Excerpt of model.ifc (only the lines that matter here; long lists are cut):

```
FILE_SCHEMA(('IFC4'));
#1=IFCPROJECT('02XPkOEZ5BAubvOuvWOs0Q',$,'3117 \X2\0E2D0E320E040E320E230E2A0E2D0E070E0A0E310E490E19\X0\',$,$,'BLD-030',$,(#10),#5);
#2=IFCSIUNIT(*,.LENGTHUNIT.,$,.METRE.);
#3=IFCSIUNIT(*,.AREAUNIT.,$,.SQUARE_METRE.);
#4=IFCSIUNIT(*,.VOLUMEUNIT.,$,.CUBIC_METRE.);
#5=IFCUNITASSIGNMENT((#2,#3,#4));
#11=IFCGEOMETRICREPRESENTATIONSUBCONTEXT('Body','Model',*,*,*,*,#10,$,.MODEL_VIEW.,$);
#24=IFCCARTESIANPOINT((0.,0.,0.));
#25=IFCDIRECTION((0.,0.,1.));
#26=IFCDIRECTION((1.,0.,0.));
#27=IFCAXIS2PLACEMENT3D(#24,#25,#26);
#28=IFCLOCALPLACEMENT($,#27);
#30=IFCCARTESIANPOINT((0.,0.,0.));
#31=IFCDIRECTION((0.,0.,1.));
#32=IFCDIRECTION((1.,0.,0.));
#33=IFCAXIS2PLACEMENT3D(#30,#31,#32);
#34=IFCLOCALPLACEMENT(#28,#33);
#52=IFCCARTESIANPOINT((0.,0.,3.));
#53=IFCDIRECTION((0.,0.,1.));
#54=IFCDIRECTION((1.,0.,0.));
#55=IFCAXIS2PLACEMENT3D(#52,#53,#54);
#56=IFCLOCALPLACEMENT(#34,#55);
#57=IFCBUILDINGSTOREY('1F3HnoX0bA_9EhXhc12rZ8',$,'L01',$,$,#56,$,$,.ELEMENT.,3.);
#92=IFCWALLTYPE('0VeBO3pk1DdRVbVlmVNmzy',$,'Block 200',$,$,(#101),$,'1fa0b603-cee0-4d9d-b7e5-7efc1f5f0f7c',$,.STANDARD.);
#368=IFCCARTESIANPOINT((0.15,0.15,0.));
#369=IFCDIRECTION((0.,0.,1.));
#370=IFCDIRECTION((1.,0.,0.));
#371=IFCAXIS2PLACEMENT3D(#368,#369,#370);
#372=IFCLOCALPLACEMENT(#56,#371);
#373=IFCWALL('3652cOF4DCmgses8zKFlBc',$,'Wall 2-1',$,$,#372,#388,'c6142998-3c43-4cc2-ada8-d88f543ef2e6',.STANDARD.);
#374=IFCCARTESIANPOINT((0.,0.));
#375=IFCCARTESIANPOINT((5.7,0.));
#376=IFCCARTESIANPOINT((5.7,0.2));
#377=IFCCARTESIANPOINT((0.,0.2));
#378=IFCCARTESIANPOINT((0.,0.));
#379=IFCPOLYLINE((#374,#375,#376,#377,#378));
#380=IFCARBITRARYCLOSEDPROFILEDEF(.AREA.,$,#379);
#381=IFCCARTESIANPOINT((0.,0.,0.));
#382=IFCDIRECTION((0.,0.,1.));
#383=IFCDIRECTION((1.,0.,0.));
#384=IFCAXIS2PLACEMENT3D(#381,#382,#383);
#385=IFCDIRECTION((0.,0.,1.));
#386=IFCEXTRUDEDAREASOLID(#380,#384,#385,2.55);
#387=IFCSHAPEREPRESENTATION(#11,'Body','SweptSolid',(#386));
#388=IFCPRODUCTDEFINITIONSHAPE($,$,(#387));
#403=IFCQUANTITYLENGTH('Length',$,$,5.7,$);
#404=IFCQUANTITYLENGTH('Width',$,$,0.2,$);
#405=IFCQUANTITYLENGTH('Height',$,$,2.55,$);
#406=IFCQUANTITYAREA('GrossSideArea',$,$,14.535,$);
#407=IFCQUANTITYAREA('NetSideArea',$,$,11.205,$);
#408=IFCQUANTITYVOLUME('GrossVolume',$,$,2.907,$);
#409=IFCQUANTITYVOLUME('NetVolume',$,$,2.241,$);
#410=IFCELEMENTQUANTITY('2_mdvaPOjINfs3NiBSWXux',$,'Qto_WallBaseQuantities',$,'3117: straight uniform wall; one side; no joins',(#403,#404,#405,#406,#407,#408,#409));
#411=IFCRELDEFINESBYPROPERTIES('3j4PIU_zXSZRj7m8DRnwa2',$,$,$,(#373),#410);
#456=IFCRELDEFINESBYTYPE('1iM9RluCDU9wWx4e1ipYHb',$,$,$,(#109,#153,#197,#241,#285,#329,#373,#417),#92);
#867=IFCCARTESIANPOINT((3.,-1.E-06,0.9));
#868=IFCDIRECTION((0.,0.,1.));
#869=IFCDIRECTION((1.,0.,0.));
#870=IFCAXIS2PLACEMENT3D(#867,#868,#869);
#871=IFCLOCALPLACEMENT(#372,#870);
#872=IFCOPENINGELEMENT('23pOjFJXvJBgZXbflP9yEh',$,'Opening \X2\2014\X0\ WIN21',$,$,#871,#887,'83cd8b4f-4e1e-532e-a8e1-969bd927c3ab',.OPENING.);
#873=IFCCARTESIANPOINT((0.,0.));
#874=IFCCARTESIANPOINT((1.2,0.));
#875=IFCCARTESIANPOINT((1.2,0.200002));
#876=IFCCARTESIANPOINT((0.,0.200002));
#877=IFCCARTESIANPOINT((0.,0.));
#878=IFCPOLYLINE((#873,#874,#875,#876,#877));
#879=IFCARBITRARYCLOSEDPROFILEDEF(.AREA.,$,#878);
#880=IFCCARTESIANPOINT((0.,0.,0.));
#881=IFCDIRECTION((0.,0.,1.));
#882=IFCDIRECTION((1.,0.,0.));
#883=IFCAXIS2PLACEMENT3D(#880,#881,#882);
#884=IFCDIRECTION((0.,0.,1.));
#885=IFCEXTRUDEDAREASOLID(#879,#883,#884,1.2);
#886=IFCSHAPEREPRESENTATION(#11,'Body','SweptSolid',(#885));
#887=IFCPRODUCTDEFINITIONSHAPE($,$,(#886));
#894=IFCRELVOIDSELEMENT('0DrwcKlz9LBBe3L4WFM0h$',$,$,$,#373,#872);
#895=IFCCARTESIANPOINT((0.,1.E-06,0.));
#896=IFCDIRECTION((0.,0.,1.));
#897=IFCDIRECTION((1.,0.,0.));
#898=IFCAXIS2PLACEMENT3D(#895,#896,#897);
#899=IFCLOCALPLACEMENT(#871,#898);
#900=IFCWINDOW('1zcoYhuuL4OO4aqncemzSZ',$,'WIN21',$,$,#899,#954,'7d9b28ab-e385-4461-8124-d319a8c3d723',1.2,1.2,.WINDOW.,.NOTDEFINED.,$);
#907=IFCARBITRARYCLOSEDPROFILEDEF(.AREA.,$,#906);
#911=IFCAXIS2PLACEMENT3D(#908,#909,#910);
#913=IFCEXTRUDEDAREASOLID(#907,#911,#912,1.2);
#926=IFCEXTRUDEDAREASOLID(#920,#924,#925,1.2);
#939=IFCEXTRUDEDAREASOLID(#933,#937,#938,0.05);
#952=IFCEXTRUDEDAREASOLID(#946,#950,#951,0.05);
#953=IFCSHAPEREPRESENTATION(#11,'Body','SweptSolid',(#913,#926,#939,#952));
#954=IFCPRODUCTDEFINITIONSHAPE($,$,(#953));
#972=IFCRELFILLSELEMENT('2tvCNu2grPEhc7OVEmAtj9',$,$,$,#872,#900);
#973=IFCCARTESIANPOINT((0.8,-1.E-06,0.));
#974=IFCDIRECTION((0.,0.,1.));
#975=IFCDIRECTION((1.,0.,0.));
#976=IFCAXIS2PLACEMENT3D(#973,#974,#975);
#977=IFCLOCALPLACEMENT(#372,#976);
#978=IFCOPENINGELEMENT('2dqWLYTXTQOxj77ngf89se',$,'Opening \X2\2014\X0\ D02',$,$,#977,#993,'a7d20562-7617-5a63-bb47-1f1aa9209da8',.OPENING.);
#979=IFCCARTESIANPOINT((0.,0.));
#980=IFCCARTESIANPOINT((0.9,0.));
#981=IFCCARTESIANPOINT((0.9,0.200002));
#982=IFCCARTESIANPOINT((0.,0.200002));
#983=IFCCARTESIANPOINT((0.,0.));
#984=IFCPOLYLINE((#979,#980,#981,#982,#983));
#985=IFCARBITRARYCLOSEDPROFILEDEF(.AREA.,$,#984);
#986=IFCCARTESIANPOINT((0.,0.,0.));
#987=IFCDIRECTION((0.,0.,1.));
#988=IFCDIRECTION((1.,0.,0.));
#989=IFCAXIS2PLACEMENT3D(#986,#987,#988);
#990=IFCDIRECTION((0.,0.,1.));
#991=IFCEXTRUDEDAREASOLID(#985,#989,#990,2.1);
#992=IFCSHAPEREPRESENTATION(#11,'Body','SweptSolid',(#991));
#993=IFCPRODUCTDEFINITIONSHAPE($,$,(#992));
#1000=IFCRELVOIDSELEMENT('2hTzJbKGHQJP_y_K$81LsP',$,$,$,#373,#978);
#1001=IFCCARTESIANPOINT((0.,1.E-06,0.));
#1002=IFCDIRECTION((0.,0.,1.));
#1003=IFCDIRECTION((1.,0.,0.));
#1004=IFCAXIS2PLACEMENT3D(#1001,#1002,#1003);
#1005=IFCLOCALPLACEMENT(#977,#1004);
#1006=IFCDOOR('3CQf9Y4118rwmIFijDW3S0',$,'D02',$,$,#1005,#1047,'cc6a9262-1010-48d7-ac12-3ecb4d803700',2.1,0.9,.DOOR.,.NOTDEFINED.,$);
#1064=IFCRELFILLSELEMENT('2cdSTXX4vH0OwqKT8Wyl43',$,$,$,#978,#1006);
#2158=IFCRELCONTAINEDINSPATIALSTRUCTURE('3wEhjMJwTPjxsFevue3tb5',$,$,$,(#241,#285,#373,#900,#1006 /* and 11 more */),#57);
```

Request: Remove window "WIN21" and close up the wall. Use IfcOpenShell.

```python
import ifcopenshell
import ifcopenshell.api.feature
import ifcopenshell.api.pset
import ifcopenshell.api.root
import ifcopenshell.geom
import ifcopenshell.util.element
import ifcopenshell.util.shape
import ifcopenshell.util.unit

model = ifcopenshell.open("model.ifc")
area_scale = ifcopenshell.util.unit.calculate_unit_scale(model, "AREAUNIT")
volume_scale = ifcopenshell.util.unit.calculate_unit_scale(model, "VOLUMEUNIT")
settings = ifcopenshell.geom.settings()


def volume(element):
    """Net volume in cubic metres, openings subtracted."""
    shape = ifcopenshell.geom.create_shape(settings, element)
    return ifcopenshell.util.shape.get_volume(shape.geometry)


window = model.by_id(900)
opening = window.FillsVoids[0].RelatingOpeningElement
wall = opening.VoidsElements[0].RelatingBuildingElement
before = volume(wall)

ifcopenshell.api.root.remove_product(model, product=window)
ifcopenshell.api.feature.remove_feature(model, feature=opening)

after = volume(wall)
thickness = 0.2  # wall thickness in metres

# Update the wall's stored quantities.
qto = model.by_id(ifcopenshell.util.element.get_pset(wall, "Qto_WallBaseQuantities", should_inherit=False)["id"])
ifcopenshell.api.pset.edit_qto(model, qto=qto, properties={
    "NetSideArea": after / thickness / area_scale,
    "NetVolume": after / volume_scale,
})

print(f"wall volume {before:.3f} -> {after:.3f} m3")

model.write("model_rev.ifc")
```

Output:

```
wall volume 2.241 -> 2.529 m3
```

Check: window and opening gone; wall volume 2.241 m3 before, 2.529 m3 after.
